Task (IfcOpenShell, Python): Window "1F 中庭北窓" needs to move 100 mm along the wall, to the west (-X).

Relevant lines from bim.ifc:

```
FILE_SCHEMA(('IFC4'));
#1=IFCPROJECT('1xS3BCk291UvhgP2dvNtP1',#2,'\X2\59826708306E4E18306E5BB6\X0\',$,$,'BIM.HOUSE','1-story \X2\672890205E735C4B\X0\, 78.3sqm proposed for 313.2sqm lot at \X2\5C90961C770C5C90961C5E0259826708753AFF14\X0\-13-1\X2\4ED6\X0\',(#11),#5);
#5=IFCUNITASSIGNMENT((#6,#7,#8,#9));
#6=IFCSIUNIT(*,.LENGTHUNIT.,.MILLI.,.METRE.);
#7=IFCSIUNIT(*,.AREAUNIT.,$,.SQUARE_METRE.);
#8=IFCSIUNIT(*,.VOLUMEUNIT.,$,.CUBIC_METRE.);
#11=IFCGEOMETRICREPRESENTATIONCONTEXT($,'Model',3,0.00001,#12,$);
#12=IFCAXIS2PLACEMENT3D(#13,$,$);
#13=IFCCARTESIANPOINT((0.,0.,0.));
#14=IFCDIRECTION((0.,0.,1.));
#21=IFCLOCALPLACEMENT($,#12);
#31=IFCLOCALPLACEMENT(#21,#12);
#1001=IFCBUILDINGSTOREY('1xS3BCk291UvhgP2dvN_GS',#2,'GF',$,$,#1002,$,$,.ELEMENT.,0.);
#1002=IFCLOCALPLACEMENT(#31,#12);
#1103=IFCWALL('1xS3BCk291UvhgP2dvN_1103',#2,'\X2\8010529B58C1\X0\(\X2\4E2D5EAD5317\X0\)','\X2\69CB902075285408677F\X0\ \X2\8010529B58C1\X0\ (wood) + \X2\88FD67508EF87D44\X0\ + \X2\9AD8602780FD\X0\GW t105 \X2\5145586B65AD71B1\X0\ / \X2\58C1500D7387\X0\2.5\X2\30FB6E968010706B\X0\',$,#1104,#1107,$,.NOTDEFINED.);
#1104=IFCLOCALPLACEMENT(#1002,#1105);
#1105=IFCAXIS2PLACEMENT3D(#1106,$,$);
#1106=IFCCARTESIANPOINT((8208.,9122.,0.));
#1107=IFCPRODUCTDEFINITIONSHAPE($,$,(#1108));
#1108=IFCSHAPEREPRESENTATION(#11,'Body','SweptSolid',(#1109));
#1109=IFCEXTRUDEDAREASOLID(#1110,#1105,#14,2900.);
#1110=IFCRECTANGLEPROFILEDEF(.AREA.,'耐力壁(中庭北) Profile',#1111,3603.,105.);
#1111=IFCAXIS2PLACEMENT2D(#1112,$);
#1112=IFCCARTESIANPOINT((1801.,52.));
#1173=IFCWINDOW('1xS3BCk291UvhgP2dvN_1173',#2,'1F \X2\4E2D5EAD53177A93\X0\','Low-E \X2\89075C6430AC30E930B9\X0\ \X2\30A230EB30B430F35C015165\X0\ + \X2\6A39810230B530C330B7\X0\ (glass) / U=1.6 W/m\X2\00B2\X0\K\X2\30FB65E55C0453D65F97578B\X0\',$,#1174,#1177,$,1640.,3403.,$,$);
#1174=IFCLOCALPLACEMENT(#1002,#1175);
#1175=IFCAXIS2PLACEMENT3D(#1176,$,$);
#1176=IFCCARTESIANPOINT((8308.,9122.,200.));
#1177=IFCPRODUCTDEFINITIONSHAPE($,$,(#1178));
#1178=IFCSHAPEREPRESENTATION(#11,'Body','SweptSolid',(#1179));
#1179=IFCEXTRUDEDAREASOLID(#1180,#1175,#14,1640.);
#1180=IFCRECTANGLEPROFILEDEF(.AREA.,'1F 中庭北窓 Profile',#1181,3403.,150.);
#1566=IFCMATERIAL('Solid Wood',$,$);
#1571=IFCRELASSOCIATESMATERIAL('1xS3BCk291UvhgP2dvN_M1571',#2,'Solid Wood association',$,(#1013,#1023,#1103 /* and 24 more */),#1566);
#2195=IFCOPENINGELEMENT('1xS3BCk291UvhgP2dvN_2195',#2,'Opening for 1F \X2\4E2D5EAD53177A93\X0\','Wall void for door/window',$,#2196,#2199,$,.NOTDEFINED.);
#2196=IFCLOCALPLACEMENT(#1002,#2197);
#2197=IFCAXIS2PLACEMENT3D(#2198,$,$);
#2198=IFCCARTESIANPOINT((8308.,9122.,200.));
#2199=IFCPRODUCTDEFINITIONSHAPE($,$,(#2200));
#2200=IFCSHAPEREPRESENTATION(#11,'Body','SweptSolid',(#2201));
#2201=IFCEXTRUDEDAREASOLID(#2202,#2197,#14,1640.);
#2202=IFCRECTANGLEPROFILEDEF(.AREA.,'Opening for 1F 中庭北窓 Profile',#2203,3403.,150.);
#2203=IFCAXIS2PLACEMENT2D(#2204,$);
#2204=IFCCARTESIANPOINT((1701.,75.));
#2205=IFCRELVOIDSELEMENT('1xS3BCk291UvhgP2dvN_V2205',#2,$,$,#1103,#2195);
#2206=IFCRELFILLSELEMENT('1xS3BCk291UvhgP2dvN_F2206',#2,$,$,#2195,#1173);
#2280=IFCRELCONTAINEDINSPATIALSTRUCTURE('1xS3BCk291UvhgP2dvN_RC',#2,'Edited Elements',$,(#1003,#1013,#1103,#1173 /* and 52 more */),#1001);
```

```python
import ifcopenshell
import ifcopenshell.api.geometry
import ifcopenshell.util.placement
import ifcopenshell.util.unit

model = ifcopenshell.open("bim.ifc")
unit_scale = ifcopenshell.util.unit.calculate_unit_scale(model)

window = model.by_guid("1xS3BCk291UvhgP2dvN_1173")
opening = window.FillsVoids[0].RelatingOpeningElement
wall = opening.VoidsElements[0].RelatingBuildingElement

wall_matrix = ifcopenshell.util.placement.get_local_placement(wall.ObjectPlacement)
shift = wall_matrix[:3, 0] * -0.1 / unit_scale
before = ifcopenshell.util.placement.get_local_placement(window.ObjectPlacement)[:3, 3].copy()

# The window is not placed relative to its opening, so move both.
for product in (opening, window):
    matrix = ifcopenshell.util.placement.get_local_placement(product.ObjectPlacement)
    matrix[:3, 3] += shift
    ifcopenshell.api.geometry.edit_object_placement(model, product=product, matrix=matrix, is_si=False)

after = ifcopenshell.util.placement.get_local_placement(window.ObjectPlacement)[:3, 3]
print("window moved by", (after - before).round(3) + 0.0)

model.write("bim_updated.ifc")
```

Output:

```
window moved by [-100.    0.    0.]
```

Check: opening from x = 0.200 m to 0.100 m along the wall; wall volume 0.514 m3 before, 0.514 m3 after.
